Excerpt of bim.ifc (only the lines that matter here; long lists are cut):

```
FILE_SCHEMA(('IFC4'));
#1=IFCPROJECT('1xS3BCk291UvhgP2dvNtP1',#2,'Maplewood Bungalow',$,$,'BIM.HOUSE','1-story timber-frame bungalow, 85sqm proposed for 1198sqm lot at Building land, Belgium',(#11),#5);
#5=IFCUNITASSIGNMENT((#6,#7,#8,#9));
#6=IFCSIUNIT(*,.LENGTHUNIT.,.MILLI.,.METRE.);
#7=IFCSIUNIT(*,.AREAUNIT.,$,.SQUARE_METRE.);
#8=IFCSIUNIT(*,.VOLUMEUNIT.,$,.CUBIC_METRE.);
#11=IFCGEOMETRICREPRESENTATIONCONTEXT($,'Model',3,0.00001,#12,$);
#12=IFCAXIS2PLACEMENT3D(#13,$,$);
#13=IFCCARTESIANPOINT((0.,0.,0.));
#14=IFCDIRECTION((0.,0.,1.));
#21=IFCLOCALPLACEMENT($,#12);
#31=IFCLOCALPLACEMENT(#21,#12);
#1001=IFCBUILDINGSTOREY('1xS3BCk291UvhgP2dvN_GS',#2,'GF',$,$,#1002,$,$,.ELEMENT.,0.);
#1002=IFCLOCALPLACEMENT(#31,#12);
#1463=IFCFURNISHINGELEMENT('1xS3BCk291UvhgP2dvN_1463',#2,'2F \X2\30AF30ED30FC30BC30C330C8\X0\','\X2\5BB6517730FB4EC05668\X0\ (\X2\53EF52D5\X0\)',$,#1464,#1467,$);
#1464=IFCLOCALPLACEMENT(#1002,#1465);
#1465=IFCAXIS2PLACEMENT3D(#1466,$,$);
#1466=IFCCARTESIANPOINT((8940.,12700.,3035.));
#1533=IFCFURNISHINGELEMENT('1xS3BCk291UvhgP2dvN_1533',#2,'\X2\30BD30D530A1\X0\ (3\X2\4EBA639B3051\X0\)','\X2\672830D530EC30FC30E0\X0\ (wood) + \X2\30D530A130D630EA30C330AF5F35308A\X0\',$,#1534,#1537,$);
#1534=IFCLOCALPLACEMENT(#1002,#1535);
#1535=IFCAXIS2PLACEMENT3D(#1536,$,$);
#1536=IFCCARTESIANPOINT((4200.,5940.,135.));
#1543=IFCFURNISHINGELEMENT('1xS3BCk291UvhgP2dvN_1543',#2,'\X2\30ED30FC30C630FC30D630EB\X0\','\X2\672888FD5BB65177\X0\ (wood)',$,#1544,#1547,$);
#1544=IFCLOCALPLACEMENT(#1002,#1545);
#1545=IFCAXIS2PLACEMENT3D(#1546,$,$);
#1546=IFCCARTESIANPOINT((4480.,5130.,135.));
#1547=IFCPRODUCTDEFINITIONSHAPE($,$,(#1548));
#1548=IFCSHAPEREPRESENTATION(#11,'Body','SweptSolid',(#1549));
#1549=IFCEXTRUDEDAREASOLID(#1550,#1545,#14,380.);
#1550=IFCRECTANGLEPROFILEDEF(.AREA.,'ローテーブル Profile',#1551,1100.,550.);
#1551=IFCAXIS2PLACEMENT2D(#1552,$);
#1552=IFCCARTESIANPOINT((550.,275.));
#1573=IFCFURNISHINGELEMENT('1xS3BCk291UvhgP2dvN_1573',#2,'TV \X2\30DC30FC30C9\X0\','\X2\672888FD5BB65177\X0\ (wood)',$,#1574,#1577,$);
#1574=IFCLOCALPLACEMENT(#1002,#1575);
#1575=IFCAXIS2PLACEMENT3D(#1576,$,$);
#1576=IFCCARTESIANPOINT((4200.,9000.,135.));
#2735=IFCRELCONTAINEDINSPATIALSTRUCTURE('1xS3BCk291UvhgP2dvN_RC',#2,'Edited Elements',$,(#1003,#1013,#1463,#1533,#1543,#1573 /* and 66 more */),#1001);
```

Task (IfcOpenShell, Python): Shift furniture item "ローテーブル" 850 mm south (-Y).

```python
import ifcopenshell
import ifcopenshell.api.geometry
import ifcopenshell.util.placement
import ifcopenshell.util.unit

model = ifcopenshell.open("bim.ifc")
unit_scale = ifcopenshell.util.unit.calculate_unit_scale(model)

item = model.by_id(1543)
matrix = ifcopenshell.util.placement.get_local_placement(item.ObjectPlacement)
matrix[1, 3] -= 0.85 / unit_scale
ifcopenshell.api.geometry.edit_object_placement(model, product=item, matrix=matrix, is_si=False)

print(ifcopenshell.util.placement.get_local_placement(item.ObjectPlacement).round(3) + 0.0)

model.write("bim_v2.ifc")
```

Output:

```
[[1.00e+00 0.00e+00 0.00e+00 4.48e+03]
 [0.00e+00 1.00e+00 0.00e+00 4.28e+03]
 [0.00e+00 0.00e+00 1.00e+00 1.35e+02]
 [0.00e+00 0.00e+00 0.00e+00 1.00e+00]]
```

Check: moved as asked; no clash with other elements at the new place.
